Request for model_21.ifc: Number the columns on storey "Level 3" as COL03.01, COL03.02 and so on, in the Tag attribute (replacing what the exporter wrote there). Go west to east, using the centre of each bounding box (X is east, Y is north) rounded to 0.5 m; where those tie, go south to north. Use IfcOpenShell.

First a look at what the model holds.

```python
import ifcopenshell
import ifcopenshell.util.element
import ifcopenshell.util.placement

model = ifcopenshell.open("model_21.ifc")
print(model.schema)
storey = next(s for s in model.by_type("IfcBuildingStorey") if s.Name == "Level 3")
columns = [e for e in ifcopenshell.util.element.get_decomposition(storey) if e.is_a("IfcColumn")]
for e in sorted(columns, key=lambda e: e.id()):
    origin = ifcopenshell.util.placement.get_local_placement(e.ObjectPlacement)[:3, 3]
    print(e.id(), e.Tag, e.Name, origin.round(2) + 0.0, sep=" | ")
```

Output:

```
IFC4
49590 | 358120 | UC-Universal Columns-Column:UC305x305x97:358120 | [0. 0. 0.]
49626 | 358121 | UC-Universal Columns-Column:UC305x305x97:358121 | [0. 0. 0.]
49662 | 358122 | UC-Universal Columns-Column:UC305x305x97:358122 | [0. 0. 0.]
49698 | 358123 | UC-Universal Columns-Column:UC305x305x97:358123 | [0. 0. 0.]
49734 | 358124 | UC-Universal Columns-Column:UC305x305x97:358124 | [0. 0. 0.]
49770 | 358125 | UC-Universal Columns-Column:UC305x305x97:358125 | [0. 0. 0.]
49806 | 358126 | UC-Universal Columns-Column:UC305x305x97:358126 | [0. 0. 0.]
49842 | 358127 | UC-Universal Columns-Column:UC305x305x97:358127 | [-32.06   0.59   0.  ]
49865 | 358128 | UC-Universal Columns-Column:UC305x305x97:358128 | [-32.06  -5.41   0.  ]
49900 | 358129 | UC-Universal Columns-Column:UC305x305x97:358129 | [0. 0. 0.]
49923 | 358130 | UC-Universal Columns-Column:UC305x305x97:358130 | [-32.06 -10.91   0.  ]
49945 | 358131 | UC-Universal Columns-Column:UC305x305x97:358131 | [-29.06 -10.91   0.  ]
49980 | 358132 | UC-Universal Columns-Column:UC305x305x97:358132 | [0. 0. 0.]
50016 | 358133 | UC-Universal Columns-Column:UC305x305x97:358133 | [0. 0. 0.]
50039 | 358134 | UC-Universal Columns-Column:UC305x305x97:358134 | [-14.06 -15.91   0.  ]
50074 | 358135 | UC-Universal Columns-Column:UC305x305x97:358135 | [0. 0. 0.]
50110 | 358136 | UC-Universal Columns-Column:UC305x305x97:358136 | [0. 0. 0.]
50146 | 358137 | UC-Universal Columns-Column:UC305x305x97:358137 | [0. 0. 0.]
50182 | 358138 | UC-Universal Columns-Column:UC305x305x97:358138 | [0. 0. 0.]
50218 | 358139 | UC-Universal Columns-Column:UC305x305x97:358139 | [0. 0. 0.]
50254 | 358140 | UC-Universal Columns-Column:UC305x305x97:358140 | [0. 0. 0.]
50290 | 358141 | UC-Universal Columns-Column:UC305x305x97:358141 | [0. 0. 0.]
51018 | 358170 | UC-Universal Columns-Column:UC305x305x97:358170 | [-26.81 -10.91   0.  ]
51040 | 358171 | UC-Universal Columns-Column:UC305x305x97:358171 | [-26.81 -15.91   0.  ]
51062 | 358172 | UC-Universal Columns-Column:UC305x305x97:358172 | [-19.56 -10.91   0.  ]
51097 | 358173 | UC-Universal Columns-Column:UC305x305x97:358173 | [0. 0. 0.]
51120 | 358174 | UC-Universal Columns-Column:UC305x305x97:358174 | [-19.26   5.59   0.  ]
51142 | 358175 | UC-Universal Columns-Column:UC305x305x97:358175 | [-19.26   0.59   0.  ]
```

```python
import ifcopenshell
import ifcopenshell.geom
import ifcopenshell.util.element
import ifcopenshell.util.shape

model = ifcopenshell.open("model_21.ifc")
settings = ifcopenshell.geom.settings()
settings.set("use-world-coords", True)


def centre(element):
    shape = ifcopenshell.geom.create_shape(settings, element)
    return ifcopenshell.util.shape.get_bbox_centroid(shape.geometry)


storey = next(s for s in model.by_type("IfcBuildingStorey") if s.Name == "Level 3")
columns = [e for e in ifcopenshell.util.element.get_decomposition(storey) if e.is_a("IfcColumn")]

# Insertion points can sit at a corner or the storey origin, so sort by the geometry (in metres).
centres = {e: centre(e) for e in columns}
columns.sort(key=lambda e: (round(centres[e][0] / 0.5), centres[e][1]))

for i, e in enumerate(columns, start=1):
    number = f"COL03.{i:02d}"
    e.Tag = number
    print(e.id(), number)

model.write("model_21_rev.ifc")
```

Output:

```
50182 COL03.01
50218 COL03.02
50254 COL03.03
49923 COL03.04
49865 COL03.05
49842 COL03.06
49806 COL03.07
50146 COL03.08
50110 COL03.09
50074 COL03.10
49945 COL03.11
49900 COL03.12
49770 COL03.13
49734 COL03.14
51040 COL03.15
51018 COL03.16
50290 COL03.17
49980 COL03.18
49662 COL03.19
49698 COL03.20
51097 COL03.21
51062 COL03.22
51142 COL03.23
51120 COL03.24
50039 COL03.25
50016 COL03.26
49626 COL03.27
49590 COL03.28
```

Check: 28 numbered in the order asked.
